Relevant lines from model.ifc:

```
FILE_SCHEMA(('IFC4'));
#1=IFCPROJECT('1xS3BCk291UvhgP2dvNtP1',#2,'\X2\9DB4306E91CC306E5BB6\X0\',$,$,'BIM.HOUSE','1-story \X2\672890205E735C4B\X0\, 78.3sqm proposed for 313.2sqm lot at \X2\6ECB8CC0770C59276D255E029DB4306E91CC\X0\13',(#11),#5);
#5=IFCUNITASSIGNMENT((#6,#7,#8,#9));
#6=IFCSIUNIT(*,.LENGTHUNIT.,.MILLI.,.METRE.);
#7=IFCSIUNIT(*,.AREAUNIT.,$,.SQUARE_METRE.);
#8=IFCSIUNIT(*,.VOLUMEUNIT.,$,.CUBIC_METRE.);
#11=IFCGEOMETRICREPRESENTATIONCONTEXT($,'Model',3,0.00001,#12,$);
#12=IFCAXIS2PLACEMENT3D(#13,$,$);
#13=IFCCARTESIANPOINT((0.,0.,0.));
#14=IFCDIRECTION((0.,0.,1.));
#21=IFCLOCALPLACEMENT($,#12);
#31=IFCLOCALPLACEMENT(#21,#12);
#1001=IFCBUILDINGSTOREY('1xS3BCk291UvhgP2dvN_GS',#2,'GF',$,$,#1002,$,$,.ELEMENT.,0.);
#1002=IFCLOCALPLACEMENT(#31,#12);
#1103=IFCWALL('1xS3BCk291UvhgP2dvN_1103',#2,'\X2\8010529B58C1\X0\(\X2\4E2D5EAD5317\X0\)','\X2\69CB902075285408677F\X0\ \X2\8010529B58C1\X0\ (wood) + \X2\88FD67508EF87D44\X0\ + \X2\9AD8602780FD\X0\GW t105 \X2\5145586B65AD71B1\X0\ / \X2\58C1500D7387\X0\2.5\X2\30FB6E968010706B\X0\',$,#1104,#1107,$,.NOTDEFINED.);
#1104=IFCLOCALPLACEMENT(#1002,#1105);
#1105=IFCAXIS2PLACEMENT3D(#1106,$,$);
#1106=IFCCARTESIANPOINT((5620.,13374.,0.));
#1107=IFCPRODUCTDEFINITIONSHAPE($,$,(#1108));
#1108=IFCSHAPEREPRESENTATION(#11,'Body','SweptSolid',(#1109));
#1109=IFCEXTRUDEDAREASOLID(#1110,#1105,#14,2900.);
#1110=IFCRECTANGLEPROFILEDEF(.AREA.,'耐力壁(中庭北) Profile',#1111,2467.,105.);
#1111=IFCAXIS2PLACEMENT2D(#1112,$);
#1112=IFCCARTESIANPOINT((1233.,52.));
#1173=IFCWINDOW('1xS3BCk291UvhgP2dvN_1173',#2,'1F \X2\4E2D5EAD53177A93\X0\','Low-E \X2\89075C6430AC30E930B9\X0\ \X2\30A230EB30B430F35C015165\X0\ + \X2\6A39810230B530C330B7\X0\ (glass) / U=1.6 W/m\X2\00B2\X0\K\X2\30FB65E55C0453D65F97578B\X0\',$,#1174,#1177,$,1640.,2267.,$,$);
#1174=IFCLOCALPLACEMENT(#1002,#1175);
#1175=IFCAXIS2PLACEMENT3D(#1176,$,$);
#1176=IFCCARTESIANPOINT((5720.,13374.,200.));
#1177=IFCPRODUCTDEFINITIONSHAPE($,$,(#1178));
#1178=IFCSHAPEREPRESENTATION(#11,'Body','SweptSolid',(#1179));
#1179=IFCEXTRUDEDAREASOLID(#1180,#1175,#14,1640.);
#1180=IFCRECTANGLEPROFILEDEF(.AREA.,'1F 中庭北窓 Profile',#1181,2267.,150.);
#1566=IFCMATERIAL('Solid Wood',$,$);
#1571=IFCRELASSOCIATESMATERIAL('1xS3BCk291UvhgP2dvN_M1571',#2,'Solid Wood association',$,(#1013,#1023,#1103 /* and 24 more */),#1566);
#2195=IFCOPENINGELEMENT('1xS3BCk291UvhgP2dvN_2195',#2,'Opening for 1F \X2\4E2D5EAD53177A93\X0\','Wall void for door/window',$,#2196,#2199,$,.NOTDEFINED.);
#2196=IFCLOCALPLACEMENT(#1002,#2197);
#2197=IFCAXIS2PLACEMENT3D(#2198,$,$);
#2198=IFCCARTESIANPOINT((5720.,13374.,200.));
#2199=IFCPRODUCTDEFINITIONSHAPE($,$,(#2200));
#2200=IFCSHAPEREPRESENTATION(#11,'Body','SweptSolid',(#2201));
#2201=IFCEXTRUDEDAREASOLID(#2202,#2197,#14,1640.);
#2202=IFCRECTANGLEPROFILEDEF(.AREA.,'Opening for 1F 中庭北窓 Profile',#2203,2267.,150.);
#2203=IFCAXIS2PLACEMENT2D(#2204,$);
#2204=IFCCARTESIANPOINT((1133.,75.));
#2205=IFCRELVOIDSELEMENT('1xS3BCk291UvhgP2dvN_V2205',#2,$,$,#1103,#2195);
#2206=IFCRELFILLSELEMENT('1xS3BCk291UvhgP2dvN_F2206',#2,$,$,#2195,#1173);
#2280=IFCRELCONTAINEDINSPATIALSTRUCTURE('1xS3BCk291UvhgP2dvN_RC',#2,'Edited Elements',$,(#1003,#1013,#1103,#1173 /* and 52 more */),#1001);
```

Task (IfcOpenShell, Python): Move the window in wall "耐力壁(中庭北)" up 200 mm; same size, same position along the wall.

```python
import numpy as np
import ifcopenshell
import ifcopenshell.api.geometry
import ifcopenshell.util.placement
import ifcopenshell.util.unit

model = ifcopenshell.open("model.ifc")
unit_scale = ifcopenshell.util.unit.calculate_unit_scale(model)

window = model.by_guid("1xS3BCk291UvhgP2dvN_1173")
opening = window.FillsVoids[0].RelatingOpeningElement
dz = 0.2 / unit_scale

shift = np.array([0.0, 0.0, dz])
# The window is not placed relative to its opening, so move both.
for product in (opening, window):
    matrix = ifcopenshell.util.placement.get_local_placement(product.ObjectPlacement)
    matrix[:3, 3] += shift
    ifcopenshell.api.geometry.edit_object_placement(model, product=product, matrix=matrix, is_si=False)

print(f"moved by {dz * unit_scale:+.3f} m")

model.write("model_updated.ifc")
```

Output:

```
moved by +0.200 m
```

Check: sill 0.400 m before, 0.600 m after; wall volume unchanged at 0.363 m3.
